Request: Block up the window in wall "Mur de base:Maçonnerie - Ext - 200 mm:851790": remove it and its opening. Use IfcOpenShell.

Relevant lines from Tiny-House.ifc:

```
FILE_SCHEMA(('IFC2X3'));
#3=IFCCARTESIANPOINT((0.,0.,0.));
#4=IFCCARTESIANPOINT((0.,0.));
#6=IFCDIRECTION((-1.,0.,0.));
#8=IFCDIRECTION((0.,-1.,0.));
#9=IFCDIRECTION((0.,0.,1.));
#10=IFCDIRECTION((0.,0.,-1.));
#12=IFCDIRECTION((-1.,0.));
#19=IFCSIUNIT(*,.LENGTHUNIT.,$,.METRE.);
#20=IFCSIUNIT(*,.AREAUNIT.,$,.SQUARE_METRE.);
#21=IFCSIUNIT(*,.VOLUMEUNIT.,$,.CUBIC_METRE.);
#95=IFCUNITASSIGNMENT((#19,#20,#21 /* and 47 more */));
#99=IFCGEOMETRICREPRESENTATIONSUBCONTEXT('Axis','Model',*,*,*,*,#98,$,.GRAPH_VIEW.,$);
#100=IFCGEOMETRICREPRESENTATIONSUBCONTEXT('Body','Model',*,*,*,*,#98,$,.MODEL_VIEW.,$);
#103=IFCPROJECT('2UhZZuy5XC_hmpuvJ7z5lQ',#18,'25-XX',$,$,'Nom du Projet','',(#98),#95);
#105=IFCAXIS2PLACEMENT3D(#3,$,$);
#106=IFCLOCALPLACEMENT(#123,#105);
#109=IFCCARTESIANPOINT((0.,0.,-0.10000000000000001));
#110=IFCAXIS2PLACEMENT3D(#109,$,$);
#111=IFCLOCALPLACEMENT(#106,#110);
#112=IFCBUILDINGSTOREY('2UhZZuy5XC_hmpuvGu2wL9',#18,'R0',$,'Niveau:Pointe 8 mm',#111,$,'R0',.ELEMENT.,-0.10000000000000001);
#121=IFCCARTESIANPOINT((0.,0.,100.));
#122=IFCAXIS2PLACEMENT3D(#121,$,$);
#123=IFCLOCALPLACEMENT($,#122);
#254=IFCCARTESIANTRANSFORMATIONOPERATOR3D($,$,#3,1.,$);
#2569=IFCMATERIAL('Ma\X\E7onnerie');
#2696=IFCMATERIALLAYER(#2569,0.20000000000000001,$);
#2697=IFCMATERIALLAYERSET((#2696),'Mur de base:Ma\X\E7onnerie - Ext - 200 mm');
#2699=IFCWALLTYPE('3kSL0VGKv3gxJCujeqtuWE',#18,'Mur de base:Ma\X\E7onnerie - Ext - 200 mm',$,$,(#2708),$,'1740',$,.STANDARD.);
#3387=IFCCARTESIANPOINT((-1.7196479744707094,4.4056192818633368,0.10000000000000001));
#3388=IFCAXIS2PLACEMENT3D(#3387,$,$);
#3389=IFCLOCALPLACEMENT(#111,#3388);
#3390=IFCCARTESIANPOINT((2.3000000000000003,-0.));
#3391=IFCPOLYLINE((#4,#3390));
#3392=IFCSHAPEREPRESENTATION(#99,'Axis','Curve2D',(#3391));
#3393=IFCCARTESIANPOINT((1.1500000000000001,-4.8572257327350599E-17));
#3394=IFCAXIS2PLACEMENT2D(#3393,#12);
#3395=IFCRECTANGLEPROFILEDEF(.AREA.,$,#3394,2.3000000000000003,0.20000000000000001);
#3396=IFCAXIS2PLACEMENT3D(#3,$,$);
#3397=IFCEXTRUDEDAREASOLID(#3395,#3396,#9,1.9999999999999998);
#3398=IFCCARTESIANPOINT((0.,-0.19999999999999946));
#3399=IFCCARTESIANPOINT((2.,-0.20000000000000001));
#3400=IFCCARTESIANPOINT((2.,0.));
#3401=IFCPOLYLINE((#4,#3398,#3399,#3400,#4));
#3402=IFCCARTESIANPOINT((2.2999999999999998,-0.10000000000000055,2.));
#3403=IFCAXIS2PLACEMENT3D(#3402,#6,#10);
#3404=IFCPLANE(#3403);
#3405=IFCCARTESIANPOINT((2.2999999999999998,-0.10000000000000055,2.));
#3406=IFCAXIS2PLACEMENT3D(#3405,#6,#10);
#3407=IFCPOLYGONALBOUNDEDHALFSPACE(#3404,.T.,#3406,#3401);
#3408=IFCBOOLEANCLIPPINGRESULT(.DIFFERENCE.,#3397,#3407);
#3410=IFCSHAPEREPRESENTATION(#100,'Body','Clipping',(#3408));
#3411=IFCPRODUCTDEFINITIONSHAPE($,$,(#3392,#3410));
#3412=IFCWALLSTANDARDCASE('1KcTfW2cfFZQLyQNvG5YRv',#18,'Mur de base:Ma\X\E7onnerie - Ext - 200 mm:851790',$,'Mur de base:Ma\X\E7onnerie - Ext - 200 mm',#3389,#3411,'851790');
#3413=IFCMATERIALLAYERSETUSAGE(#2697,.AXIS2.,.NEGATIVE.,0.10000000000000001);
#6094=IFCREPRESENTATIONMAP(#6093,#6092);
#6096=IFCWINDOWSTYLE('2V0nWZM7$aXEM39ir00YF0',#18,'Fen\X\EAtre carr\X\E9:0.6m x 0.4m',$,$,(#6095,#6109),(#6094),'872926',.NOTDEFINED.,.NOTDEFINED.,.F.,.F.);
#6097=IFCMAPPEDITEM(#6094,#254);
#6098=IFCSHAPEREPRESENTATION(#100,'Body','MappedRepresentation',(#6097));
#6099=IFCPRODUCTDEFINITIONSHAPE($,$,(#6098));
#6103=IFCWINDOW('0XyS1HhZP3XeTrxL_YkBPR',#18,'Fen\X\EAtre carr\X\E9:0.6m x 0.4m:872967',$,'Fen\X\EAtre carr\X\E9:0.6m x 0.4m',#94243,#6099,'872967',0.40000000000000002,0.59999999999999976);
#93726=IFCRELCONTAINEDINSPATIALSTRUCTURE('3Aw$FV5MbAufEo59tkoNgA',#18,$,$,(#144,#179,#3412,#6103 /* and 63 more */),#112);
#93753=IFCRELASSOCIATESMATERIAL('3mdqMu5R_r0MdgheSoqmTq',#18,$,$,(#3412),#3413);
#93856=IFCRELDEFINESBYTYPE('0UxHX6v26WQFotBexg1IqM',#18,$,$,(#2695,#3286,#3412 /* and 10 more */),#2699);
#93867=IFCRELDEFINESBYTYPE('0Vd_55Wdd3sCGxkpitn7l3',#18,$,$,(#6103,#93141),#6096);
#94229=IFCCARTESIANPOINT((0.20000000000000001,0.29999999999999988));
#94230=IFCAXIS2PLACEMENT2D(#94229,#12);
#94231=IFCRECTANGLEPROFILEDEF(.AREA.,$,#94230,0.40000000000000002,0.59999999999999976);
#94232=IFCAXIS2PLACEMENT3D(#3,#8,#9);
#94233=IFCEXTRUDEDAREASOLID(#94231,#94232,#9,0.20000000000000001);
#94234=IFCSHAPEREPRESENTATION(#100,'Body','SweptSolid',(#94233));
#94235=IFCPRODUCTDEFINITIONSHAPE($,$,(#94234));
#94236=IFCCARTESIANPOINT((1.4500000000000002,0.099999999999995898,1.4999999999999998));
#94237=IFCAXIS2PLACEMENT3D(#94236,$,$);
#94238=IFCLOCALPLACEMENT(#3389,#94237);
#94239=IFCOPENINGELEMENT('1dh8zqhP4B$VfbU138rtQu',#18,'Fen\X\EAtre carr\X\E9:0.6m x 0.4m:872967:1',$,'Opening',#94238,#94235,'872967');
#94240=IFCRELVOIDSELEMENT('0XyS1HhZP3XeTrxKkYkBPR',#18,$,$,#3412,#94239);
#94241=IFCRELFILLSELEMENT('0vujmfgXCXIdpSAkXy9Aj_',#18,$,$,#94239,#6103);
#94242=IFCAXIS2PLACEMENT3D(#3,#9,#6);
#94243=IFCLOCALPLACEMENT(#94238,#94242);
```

```python
import ifcopenshell
import ifcopenshell.api.feature
import ifcopenshell.api.root
import ifcopenshell.geom
import ifcopenshell.util.shape

model = ifcopenshell.open("Tiny-House.ifc")
settings = ifcopenshell.geom.settings()


def volume(element):
    """Net volume in cubic metres, openings subtracted."""
    shape = ifcopenshell.geom.create_shape(settings, element)
    return ifcopenshell.util.shape.get_volume(shape.geometry)


window = model.by_guid("0XyS1HhZP3XeTrxL_YkBPR")
opening = window.FillsVoids[0].RelatingOpeningElement
wall = opening.VoidsElements[0].RelatingBuildingElement
before = volume(wall)

ifcopenshell.api.root.remove_product(model, product=window)
ifcopenshell.api.feature.remove_feature(model, feature=opening)

after = volume(wall)

print(f"wall volume {before:.3f} -> {after:.3f} m3")

model.write("Tiny-House_v2.ifc")
```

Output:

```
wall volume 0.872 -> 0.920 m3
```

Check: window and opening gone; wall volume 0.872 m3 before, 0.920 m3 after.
